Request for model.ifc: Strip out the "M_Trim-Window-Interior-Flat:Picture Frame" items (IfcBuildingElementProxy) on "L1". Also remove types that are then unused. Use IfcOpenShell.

First a look at what the model holds.

```python
import ifcopenshell
import ifcopenshell.util.element

model = ifcopenshell.open("model.ifc")
print(model.schema)
storey = next(s for s in model.by_type("IfcBuildingStorey") if s.Name == "L1")
proxies = [e for e in ifcopenshell.util.element.get_decomposition(storey) if e.is_a("IfcBuildingElementProxy")]
seen = {}
for e in proxies:
    element_type = ifcopenshell.util.element.get_type(e)
    name = element_type.Name if element_type not in (None, e) else None
    seen[name] = seen.get(name, 0) + 1
for name, count in sorted(seen.items(), key=str):
    print(count, "x", name)
```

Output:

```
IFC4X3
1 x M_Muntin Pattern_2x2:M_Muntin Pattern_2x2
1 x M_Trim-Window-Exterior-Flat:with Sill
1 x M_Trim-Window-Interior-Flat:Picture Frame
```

```python
import ifcopenshell
import ifcopenshell.api.root
import ifcopenshell.util.element

model = ifcopenshell.open("model.ifc")

storey = next(s for s in model.by_type("IfcBuildingStorey") if s.Name == "L1")
proxies = [e for e in ifcopenshell.util.element.get_decomposition(storey) if e.is_a("IfcBuildingElementProxy")]
targets = [e for e in proxies if (t := ifcopenshell.util.element.get_type(e)) not in (None, e) and t.Name == "M_Trim-Window-Interior-Flat:Picture Frame"]
types = {ifcopenshell.util.element.get_type(e) for e in targets} - {None, *targets}

for e in targets:
    ifcopenshell.api.root.remove_product(model, product=e)
print(len(targets), "removed")

unused = [t for t in types if not ifcopenshell.util.element.get_types(t)]
for t in unused:
    ifcopenshell.api.root.remove_product(model, product=t)
print(len(unused), "unused types removed")

model.write("model_updated.ifc")
```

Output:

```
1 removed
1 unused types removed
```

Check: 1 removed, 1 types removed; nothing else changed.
